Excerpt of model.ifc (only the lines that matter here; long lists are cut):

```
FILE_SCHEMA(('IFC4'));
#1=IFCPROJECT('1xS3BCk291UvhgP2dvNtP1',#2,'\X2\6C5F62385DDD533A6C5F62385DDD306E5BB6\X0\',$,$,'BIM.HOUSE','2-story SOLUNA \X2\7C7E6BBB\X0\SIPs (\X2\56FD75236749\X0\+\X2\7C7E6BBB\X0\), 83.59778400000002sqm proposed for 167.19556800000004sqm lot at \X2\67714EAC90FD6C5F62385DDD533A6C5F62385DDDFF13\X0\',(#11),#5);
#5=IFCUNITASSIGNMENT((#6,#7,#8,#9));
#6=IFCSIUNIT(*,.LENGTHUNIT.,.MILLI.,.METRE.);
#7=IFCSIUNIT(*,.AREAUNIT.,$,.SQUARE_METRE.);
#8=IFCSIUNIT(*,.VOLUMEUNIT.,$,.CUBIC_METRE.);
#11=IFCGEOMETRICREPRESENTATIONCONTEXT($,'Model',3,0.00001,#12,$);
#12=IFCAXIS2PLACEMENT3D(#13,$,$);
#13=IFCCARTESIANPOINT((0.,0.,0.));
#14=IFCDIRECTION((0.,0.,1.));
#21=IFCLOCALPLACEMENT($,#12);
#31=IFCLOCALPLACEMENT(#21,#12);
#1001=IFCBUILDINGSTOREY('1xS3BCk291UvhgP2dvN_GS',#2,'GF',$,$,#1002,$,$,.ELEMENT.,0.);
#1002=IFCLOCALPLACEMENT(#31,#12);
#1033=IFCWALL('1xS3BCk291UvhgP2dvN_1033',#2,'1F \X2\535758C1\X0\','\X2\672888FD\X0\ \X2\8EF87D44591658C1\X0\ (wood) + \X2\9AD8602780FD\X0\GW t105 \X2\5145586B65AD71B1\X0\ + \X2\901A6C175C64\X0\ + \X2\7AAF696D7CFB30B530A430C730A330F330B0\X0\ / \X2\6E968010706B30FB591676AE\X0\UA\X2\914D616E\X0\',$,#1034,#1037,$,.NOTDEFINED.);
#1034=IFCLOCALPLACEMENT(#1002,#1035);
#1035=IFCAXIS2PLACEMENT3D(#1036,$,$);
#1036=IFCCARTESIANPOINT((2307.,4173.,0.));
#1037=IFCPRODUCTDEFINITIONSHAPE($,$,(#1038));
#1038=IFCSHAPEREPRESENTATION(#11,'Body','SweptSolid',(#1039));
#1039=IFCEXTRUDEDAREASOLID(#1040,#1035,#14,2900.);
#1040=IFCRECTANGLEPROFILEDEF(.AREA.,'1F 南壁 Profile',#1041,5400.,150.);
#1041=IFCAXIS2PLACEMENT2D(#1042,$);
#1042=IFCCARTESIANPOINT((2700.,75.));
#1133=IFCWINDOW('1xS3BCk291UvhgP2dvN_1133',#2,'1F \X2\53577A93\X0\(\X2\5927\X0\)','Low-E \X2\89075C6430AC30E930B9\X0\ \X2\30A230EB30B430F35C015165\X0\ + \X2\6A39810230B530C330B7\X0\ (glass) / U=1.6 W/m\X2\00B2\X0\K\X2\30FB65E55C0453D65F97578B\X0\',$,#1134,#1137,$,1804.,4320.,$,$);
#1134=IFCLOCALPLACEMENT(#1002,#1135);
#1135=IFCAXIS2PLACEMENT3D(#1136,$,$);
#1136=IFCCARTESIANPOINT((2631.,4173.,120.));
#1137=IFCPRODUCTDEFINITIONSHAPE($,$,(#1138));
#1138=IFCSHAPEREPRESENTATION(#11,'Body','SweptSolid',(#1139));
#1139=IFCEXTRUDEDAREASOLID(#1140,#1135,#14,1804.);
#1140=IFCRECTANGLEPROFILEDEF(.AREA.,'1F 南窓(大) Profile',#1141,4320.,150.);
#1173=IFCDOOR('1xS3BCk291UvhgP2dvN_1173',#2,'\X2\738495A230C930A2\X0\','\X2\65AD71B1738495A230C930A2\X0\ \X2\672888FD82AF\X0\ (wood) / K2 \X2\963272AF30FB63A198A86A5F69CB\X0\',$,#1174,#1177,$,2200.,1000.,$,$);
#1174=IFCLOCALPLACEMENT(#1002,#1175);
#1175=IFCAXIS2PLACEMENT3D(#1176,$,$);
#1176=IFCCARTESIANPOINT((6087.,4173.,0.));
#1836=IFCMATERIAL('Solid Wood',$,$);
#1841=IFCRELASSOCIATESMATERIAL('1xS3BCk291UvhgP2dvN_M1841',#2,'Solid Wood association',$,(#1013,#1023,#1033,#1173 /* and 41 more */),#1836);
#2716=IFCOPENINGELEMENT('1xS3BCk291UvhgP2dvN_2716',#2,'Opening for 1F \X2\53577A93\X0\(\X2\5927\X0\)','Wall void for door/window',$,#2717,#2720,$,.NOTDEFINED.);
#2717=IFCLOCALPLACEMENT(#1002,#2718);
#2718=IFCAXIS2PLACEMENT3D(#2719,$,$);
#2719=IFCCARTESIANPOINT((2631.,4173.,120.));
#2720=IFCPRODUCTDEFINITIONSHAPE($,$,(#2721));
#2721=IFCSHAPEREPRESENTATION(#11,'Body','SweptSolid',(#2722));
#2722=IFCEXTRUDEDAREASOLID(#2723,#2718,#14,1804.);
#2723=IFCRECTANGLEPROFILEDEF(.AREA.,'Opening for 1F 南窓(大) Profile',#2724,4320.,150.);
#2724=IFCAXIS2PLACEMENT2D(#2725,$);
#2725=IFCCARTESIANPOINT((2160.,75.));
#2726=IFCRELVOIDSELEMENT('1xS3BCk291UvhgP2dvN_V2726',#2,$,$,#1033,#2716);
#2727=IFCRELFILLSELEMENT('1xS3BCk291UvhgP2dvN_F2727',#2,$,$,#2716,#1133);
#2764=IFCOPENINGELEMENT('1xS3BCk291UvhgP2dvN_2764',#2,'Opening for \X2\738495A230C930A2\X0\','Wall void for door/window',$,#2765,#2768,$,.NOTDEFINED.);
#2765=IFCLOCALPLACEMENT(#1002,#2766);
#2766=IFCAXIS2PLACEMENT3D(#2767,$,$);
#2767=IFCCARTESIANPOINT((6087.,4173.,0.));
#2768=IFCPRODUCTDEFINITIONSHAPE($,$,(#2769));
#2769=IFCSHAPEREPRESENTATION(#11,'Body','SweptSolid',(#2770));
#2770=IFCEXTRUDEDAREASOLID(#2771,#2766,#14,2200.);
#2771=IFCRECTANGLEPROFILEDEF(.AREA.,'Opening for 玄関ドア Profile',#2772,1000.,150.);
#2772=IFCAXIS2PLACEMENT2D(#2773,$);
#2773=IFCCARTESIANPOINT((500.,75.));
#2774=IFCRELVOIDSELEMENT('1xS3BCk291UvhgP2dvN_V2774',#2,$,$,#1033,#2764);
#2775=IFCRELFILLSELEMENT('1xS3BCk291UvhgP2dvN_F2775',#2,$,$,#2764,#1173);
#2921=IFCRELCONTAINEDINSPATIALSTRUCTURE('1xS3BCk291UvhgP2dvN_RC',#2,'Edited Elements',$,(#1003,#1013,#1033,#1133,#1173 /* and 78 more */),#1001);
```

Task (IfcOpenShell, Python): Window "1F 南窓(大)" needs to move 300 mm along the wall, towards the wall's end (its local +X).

```python
import ifcopenshell
import ifcopenshell.api.geometry
import ifcopenshell.util.placement
import ifcopenshell.util.unit

model = ifcopenshell.open("model.ifc")
unit_scale = ifcopenshell.util.unit.calculate_unit_scale(model)

window = model.by_guid("1xS3BCk291UvhgP2dvN_1133")
opening = window.FillsVoids[0].RelatingOpeningElement
wall = opening.VoidsElements[0].RelatingBuildingElement

wall_matrix = ifcopenshell.util.placement.get_local_placement(wall.ObjectPlacement)
shift = wall_matrix[:3, 0] * 0.3 / unit_scale
before = ifcopenshell.util.placement.get_local_placement(window.ObjectPlacement)[:3, 3].copy()

# The window is not placed relative to its opening, so move both.
for product in (opening, window):
    matrix = ifcopenshell.util.placement.get_local_placement(product.ObjectPlacement)
    matrix[:3, 3] += shift
    ifcopenshell.api.geometry.edit_object_placement(model, product=product, matrix=matrix, is_si=False)

after = ifcopenshell.util.placement.get_local_placement(window.ObjectPlacement)[:3, 3]
print("window moved by", (after - before).round(3) + 0.0)

model.write("model_edited.ifc")
```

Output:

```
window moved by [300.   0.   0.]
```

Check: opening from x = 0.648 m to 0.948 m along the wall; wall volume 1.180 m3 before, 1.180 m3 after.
